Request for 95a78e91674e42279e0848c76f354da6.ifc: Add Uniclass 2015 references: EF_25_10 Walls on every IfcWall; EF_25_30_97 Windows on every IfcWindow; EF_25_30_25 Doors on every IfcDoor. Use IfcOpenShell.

First a look at what the model holds.

```python
import ifcopenshell

model = ifcopenshell.open("95a78e91674e42279e0848c76f354da6.ifc")
print(model.schema)
print("classifications:", [c.Name for c in model.by_type("IfcClassification")])
for ifc_class in ("IfcDoor", "IfcRoof", "IfcStair", "IfcWall", "IfcWindow"):
    print(ifc_class, len(model.by_type(ifc_class)))
```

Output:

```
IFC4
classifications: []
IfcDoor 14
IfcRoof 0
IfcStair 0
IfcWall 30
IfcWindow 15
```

```python
import ifcopenshell
import ifcopenshell.api.classification

model = ifcopenshell.open("95a78e91674e42279e0848c76f354da6.ifc")

system = ifcopenshell.api.classification.add_classification(model, classification="Uniclass 2015")

codes = {
    "IfcWall": ("EF_25_10", "Walls"),
    "IfcWindow": ("EF_25_30_97", "Windows"),
    "IfcDoor": ("EF_25_30_25", "Doors"),
}
for ifc_class, (code, name) in codes.items():
    products = model.by_type(ifc_class)
    ifcopenshell.api.classification.add_reference(
        model, products=products, classification=system, identification=code, name=name
    )
    print(code, len(products))

model.write("95a78e91674e42279e0848c76f354da6_edited.ifc")
```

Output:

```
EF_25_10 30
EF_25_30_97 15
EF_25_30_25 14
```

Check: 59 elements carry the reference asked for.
